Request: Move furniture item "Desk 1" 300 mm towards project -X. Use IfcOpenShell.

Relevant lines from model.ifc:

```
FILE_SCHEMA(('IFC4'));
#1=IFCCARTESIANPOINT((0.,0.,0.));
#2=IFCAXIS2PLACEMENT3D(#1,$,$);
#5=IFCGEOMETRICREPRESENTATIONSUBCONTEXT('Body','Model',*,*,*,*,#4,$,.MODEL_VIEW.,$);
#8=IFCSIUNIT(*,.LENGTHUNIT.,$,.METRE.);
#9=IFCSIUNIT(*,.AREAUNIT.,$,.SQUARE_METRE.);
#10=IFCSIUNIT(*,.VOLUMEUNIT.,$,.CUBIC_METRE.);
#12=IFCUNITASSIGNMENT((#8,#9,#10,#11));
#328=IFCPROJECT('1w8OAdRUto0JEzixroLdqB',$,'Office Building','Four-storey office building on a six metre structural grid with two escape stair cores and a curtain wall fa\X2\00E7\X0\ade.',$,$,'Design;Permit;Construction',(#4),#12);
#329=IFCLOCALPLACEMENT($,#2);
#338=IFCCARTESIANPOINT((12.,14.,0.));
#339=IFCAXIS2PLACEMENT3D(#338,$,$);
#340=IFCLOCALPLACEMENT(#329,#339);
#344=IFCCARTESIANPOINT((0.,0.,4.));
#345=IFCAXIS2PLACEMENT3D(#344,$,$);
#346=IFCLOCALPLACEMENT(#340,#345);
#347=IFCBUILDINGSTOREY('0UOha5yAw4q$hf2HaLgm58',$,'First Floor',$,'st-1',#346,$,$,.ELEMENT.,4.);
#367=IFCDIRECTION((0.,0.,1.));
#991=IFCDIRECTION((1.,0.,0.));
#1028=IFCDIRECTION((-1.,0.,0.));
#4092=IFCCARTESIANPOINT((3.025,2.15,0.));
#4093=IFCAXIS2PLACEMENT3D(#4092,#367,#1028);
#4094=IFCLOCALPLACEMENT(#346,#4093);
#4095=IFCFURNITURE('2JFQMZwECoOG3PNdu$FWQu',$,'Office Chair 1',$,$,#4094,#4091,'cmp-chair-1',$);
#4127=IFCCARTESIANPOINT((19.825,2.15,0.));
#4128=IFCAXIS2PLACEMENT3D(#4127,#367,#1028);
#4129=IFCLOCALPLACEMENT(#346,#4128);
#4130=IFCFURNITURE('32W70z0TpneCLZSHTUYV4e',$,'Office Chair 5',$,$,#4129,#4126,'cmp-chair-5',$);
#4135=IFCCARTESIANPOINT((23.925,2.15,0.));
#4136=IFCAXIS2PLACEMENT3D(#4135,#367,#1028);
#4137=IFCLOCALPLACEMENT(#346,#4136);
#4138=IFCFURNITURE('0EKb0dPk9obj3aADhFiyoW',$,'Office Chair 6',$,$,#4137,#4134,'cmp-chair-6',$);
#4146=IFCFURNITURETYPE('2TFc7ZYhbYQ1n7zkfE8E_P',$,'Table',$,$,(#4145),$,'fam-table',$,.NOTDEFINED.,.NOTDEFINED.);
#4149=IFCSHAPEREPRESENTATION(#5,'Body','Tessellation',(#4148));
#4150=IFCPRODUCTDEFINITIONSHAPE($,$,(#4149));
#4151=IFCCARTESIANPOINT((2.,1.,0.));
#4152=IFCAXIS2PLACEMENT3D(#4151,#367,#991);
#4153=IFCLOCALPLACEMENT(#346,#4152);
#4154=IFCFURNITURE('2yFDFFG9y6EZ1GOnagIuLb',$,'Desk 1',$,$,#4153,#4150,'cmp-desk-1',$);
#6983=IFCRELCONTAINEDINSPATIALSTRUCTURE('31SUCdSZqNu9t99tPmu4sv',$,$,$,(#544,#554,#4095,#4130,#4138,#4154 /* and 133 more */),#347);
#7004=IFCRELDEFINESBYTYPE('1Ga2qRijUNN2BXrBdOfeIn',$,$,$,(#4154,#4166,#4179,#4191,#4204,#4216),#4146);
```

```python
import ifcopenshell
import ifcopenshell.api.geometry
import ifcopenshell.util.placement
import ifcopenshell.util.unit

model = ifcopenshell.open("model.ifc")
unit_scale = ifcopenshell.util.unit.calculate_unit_scale(model)

item = model.by_guid("2yFDFFG9y6EZ1GOnagIuLb")
matrix = ifcopenshell.util.placement.get_local_placement(item.ObjectPlacement)
matrix[0, 3] -= 0.3 / unit_scale
ifcopenshell.api.geometry.edit_object_placement(model, product=item, matrix=matrix, is_si=False)

print(ifcopenshell.util.placement.get_local_placement(item.ObjectPlacement).round(3) + 0.0)

model.write("model-out.ifc")
```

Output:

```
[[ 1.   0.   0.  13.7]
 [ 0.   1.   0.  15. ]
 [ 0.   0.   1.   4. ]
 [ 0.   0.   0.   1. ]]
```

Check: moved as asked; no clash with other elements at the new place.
